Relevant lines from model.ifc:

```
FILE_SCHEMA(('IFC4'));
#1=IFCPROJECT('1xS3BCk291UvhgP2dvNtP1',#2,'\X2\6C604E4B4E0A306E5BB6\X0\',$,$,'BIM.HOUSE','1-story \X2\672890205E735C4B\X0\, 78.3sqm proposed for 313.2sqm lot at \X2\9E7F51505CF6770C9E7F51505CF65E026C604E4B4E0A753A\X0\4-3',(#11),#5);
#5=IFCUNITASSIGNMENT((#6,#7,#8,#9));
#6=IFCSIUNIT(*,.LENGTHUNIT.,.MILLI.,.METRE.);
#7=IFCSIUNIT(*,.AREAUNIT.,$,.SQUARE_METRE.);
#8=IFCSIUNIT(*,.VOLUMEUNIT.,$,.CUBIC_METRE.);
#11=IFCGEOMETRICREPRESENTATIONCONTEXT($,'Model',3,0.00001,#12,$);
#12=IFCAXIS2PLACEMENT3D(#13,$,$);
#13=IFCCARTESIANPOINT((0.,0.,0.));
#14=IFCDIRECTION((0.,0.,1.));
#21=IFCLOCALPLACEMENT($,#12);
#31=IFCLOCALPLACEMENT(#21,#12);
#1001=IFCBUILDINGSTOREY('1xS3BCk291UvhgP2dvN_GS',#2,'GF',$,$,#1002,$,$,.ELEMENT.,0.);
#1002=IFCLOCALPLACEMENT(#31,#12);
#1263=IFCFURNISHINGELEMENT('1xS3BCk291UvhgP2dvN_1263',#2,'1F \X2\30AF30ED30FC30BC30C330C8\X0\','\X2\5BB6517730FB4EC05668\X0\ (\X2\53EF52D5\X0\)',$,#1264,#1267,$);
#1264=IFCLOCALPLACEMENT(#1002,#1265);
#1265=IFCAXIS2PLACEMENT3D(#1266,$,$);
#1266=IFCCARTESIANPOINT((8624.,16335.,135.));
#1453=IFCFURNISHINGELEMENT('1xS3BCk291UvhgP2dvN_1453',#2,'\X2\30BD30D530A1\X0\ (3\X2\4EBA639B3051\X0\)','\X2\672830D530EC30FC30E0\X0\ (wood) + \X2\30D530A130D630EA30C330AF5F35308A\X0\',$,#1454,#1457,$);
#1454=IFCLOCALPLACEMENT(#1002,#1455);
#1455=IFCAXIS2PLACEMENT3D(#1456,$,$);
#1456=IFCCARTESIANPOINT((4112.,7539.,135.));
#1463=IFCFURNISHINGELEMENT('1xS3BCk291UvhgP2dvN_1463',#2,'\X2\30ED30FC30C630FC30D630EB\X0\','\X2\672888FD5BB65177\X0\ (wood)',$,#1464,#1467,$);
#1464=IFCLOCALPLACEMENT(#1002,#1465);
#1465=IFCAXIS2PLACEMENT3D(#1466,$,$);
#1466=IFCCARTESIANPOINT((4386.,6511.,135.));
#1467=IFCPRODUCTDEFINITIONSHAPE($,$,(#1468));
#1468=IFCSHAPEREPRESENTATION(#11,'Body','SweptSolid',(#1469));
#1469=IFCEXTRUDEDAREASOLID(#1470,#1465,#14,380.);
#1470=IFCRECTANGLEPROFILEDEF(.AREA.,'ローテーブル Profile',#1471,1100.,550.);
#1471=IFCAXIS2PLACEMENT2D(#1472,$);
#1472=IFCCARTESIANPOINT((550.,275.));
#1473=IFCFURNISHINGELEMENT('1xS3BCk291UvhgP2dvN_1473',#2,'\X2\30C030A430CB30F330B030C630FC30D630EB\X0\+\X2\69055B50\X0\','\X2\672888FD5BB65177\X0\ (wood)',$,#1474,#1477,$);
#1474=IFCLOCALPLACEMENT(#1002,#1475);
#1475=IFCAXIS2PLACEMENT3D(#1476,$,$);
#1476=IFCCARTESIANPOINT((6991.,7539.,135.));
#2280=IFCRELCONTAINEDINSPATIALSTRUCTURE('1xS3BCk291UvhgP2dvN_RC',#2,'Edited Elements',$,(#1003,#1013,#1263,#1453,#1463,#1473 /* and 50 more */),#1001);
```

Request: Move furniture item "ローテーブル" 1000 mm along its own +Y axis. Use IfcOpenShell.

```python
import ifcopenshell
import ifcopenshell.api.geometry
import ifcopenshell.util.placement

model = ifcopenshell.open("model.ifc")

item = model.by_guid("1xS3BCk291UvhgP2dvN_1463")
matrix = ifcopenshell.util.placement.get_local_placement(item.ObjectPlacement)
matrix[:3, 3] += matrix[:3, 1] * 1000.0
ifcopenshell.api.geometry.edit_object_placement(model, product=item, matrix=matrix, is_si=False)

print(ifcopenshell.util.placement.get_local_placement(item.ObjectPlacement).round(3) + 0.0)

model.write("model_v2.ifc")
```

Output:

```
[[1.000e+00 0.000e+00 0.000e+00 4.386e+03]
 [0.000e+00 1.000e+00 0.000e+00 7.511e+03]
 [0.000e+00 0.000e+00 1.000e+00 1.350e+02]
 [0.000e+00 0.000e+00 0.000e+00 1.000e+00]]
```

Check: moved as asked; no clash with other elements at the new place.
